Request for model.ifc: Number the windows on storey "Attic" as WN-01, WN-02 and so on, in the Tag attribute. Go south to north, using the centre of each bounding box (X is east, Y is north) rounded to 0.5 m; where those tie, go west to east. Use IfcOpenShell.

First a look at what the model holds.

```python
import ifcopenshell
import ifcopenshell.util.element
import ifcopenshell.util.placement

model = ifcopenshell.open("model.ifc")
print(model.schema)
storey = next(s for s in model.by_type("IfcBuildingStorey") if s.Name == "Attic")
windows = [e for e in ifcopenshell.util.element.get_decomposition(storey) if e.is_a("IfcWindow")]
for e in sorted(windows, key=lambda e: e.id()):
    origin = ifcopenshell.util.placement.get_local_placement(e.ObjectPlacement)[:3, 3]
    print(e.id(), e.Tag, e.Name, origin.round(2) + 0.0, sep=" | ")
```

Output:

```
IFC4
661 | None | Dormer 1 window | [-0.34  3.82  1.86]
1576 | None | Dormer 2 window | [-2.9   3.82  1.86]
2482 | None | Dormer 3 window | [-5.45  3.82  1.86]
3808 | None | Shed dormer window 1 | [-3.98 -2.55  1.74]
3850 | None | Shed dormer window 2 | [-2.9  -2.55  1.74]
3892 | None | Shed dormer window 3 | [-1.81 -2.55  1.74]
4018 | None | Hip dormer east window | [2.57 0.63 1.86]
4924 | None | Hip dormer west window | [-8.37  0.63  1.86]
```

```python
import ifcopenshell
import ifcopenshell.geom
import ifcopenshell.util.element
import ifcopenshell.util.shape

model = ifcopenshell.open("model.ifc")
settings = ifcopenshell.geom.settings()
settings.set("use-world-coords", True)


def centre(element):
    shape = ifcopenshell.geom.create_shape(settings, element)
    return ifcopenshell.util.shape.get_bbox_centroid(shape.geometry)


storey = next(s for s in model.by_type("IfcBuildingStorey") if s.Name == "Attic")
windows = [e for e in ifcopenshell.util.element.get_decomposition(storey) if e.is_a("IfcWindow")]

# Insertion points can sit at a corner or the storey origin, so sort by the geometry (in metres).
centres = {e: centre(e) for e in windows}
windows.sort(key=lambda e: (round(centres[e][1] / 0.5), centres[e][0]))

for i, e in enumerate(windows, start=1):
    number = f"WN-{i:02d}"
    e.Tag = number
    print(e.id(), number)

model.write("model-out.ifc")
```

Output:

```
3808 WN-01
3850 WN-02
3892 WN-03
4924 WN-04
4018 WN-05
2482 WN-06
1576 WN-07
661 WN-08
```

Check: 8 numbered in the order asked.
